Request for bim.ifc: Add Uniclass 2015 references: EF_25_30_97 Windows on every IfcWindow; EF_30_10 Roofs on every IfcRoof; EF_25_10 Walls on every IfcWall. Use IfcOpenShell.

First a look at what the model holds.

```python
import ifcopenshell

model = ifcopenshell.open("bim.ifc")
print(model.schema)
print("classifications:", [c.Name for c in model.by_type("IfcClassification")])
for ifc_class in ("IfcDoor", "IfcRoof", "IfcStair", "IfcWall", "IfcWindow"):
    print(ifc_class, len(model.by_type(ifc_class)))
```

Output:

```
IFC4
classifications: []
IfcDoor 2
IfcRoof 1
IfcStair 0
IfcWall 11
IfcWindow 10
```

```python
import ifcopenshell
import ifcopenshell.api.classification

model = ifcopenshell.open("bim.ifc")

system = ifcopenshell.api.classification.add_classification(model, classification="Uniclass 2015")

codes = {
    "IfcWindow": ("EF_25_30_97", "Windows"),
    "IfcRoof": ("EF_30_10", "Roofs"),
    "IfcWall": ("EF_25_10", "Walls"),
}
for ifc_class, (code, name) in codes.items():
    products = model.by_type(ifc_class)
    ifcopenshell.api.classification.add_reference(
        model, products=products, classification=system, identification=code, name=name
    )
    print(code, len(products))

model.write("bim_v2.ifc")
```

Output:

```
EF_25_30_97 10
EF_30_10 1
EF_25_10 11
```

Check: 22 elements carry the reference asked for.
